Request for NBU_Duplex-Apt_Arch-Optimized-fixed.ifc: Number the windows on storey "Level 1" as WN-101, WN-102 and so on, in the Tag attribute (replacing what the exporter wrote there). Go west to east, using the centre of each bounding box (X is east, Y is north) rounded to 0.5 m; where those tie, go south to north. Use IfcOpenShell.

First a look at what the model holds.

```python
import ifcopenshell
import ifcopenshell.util.element
import ifcopenshell.util.placement

model = ifcopenshell.open("NBU_Duplex-Apt_Arch-Optimized-fixed.ifc")
print(model.schema)
storey = next(s for s in model.by_type("IfcBuildingStorey") if s.Name == "Level 1")
windows = [e for e in ifcopenshell.util.element.get_decomposition(storey) if e.is_a("IfcWindow")]
for e in sorted(windows, key=lambda e: e.id()):
    origin = ifcopenshell.util.placement.get_local_placement(e.ObjectPlacement)[:3, 3]
    print(e.id(), e.Tag, e.Name, origin.round(2) + 0.0, sep=" | ")
```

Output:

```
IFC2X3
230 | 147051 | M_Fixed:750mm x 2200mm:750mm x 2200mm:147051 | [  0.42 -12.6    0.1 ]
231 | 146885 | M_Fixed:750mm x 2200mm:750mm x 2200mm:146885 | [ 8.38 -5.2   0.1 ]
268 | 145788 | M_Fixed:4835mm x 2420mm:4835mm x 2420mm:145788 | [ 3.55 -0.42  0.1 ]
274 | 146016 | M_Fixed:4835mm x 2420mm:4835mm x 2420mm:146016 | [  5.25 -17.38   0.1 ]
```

```python
import ifcopenshell
import ifcopenshell.geom
import ifcopenshell.util.element
import ifcopenshell.util.shape

model = ifcopenshell.open("NBU_Duplex-Apt_Arch-Optimized-fixed.ifc")
settings = ifcopenshell.geom.settings()
settings.set("use-world-coords", True)


def centre(element):
    shape = ifcopenshell.geom.create_shape(settings, element)
    return ifcopenshell.util.shape.get_bbox_centroid(shape.geometry)


storey = next(s for s in model.by_type("IfcBuildingStorey") if s.Name == "Level 1")
windows = [e for e in ifcopenshell.util.element.get_decomposition(storey) if e.is_a("IfcWindow")]

# Insertion points can sit at a corner or the storey origin, so sort by the geometry (in metres).
centres = {e: centre(e) for e in windows}
windows.sort(key=lambda e: (round(centres[e][0] / 0.5), centres[e][1]))

for i, e in enumerate(windows, start=1):
    number = f"WN-1{i:02d}"
    e.Tag = number
    print(e.id(), number)

model.write("NBU_Duplex-Apt_Arch-Optimized-fixed_rev.ifc")
```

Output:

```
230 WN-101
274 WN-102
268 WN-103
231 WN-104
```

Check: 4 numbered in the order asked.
